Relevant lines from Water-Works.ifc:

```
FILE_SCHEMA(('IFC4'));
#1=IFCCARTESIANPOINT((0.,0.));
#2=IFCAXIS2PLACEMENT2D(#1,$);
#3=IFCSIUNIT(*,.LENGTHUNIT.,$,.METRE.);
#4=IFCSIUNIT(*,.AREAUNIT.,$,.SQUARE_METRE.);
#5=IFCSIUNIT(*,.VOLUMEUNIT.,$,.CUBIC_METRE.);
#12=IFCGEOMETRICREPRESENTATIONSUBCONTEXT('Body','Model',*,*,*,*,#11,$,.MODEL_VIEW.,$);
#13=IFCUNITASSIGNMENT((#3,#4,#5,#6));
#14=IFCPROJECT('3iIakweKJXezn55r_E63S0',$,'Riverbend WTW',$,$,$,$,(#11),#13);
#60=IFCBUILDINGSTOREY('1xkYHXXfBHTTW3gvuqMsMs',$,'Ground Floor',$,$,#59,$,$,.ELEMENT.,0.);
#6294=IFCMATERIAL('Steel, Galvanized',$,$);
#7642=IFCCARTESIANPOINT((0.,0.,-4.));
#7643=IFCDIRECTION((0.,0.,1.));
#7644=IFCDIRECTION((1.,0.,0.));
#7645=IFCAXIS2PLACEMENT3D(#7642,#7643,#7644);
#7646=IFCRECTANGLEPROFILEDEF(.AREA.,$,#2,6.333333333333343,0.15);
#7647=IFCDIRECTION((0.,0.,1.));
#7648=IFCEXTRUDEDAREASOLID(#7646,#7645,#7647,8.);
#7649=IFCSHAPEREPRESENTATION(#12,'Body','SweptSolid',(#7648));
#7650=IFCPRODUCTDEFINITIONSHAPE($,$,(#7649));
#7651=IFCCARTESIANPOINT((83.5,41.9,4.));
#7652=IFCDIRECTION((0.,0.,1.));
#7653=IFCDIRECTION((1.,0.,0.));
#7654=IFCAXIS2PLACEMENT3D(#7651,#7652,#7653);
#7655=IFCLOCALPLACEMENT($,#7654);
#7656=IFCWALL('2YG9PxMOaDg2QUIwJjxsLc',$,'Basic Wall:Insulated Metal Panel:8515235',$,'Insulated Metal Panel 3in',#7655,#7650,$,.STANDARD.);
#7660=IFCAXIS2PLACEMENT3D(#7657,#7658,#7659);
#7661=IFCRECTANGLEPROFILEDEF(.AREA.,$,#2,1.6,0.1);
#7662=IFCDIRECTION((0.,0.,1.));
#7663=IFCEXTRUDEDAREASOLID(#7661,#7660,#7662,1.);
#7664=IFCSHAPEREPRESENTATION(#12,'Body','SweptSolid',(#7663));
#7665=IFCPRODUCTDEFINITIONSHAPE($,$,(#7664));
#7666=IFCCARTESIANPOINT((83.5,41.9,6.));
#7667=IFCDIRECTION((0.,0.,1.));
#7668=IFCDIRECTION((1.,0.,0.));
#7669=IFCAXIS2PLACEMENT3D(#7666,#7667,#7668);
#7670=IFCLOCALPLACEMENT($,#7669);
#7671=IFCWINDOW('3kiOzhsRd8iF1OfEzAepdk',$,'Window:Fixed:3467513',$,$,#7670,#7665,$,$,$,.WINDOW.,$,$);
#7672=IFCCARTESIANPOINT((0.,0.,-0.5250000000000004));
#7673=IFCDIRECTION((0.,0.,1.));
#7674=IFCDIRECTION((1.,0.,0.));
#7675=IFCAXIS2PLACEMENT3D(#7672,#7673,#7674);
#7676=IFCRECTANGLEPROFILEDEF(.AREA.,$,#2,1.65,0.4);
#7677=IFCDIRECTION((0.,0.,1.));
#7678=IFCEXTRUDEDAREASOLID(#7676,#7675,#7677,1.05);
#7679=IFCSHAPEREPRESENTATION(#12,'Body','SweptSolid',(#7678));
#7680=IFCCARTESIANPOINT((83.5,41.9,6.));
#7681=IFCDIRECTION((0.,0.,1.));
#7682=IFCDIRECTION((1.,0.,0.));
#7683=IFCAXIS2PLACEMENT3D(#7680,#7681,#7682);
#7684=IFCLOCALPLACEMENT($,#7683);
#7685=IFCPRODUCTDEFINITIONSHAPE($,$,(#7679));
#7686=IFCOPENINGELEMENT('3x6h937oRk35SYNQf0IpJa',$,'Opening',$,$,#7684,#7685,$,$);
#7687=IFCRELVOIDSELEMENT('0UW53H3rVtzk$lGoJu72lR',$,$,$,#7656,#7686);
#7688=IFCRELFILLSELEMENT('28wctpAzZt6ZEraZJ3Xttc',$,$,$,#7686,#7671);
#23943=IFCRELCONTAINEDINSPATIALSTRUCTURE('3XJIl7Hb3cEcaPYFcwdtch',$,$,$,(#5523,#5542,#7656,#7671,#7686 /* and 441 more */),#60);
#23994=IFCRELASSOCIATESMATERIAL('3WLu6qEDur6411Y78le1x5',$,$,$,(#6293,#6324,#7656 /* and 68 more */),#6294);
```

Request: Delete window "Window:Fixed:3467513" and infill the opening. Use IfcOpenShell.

```python
import ifcopenshell
import ifcopenshell.api.feature
import ifcopenshell.api.root
import ifcopenshell.geom
import ifcopenshell.util.shape

model = ifcopenshell.open("Water-Works.ifc")
settings = ifcopenshell.geom.settings()


def volume(element):
    """Net volume in cubic metres, openings subtracted."""
    shape = ifcopenshell.geom.create_shape(settings, element)
    return ifcopenshell.util.shape.get_volume(shape.geometry)


window = model.by_guid("3kiOzhsRd8iF1OfEzAepdk")
opening = window.FillsVoids[0].RelatingOpeningElement
wall = opening.VoidsElements[0].RelatingBuildingElement
before = volume(wall)

ifcopenshell.api.root.remove_product(model, product=window)
ifcopenshell.api.feature.remove_feature(model, feature=opening)

after = volume(wall)

print(f"wall volume {before:.3f} -> {after:.3f} m3")

model.write("Water-Works_v2.ifc")
```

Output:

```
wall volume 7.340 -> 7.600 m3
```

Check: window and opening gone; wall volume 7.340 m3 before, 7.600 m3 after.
